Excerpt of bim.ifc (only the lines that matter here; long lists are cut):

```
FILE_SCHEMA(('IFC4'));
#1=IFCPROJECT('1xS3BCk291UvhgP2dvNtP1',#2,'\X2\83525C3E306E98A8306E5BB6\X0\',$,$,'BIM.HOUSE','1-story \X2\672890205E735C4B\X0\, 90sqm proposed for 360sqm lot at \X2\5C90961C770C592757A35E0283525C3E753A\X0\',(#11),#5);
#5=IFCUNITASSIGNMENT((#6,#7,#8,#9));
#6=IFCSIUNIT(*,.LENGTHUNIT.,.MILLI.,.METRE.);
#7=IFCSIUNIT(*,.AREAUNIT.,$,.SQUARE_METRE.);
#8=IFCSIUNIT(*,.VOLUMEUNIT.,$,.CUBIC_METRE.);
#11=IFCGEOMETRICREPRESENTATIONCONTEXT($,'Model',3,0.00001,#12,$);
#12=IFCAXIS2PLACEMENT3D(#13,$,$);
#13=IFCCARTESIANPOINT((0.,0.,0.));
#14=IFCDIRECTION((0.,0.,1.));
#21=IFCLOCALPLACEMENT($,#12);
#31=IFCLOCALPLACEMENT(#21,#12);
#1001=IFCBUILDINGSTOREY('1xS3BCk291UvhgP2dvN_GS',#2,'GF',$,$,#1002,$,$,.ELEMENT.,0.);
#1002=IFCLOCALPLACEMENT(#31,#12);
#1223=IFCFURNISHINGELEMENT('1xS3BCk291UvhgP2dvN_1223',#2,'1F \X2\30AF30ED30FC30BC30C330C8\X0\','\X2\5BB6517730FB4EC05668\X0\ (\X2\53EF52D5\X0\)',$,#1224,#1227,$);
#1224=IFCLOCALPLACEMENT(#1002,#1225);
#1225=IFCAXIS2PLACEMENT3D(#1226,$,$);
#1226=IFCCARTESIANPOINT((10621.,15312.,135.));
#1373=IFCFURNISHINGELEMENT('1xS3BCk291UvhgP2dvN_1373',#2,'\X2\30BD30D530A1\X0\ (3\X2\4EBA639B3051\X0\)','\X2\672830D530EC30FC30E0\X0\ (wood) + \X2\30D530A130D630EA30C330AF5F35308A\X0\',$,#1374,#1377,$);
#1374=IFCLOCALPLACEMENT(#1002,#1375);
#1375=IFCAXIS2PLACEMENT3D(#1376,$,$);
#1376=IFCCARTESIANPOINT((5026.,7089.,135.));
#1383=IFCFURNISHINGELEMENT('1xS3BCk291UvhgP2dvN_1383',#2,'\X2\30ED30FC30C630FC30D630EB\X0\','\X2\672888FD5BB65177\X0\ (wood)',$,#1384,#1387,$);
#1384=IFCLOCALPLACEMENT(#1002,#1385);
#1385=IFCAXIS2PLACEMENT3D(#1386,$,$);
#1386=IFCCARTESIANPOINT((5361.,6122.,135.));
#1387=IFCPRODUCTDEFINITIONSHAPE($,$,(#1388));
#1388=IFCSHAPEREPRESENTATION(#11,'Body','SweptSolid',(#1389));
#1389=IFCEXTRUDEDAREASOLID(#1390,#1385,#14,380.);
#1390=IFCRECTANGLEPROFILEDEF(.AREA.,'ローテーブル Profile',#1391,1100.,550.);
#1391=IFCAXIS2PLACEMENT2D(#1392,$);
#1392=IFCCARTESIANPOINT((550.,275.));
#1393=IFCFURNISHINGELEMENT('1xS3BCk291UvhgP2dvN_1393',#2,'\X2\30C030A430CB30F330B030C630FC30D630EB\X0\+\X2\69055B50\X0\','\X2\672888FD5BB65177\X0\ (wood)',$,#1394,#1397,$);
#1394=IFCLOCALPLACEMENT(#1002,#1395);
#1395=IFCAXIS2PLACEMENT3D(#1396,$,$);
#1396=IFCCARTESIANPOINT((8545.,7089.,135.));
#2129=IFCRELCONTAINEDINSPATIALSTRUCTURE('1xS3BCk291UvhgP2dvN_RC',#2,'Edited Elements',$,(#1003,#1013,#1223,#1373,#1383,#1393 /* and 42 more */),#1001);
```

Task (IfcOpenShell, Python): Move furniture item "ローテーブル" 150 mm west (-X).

```python
import ifcopenshell
import ifcopenshell.api.geometry
import ifcopenshell.util.placement

model = ifcopenshell.open("bim.ifc")

item = model.by_id(1383)
matrix = ifcopenshell.util.placement.get_local_placement(item.ObjectPlacement)
matrix[0, 3] -= 150.0
ifcopenshell.api.geometry.edit_object_placement(model, product=item, matrix=matrix, is_si=False)

print(ifcopenshell.util.placement.get_local_placement(item.ObjectPlacement).round(3) + 0.0)

model.write("bim_updated.ifc")
```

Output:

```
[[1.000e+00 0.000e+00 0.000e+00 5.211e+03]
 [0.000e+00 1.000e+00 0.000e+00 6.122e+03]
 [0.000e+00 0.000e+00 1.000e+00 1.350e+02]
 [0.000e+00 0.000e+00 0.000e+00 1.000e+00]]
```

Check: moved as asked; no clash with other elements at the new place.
